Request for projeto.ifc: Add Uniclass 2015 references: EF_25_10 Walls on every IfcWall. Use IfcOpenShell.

First a look at what the model holds.

```python
import ifcopenshell

model = ifcopenshell.open("projeto.ifc")
print(model.schema)
print("classifications:", [c.Name for c in model.by_type("IfcClassification")])
for ifc_class in ("IfcDoor", "IfcRoof", "IfcStair", "IfcWall", "IfcWindow"):
    print(ifc_class, len(model.by_type(ifc_class)))
```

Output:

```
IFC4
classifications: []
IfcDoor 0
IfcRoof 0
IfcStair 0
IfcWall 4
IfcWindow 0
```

```python
import ifcopenshell
import ifcopenshell.api.classification

model = ifcopenshell.open("projeto.ifc")

system = ifcopenshell.api.classification.add_classification(model, classification="Uniclass 2015")

codes = {
    "IfcWall": ("EF_25_10", "Walls"),
}
for ifc_class, (code, name) in codes.items():
    products = model.by_type(ifc_class)
    ifcopenshell.api.classification.add_reference(
        model, products=products, classification=system, identification=code, name=name
    )
    print(code, len(products))

model.write("projeto_rev.ifc")
```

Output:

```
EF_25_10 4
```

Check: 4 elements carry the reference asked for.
